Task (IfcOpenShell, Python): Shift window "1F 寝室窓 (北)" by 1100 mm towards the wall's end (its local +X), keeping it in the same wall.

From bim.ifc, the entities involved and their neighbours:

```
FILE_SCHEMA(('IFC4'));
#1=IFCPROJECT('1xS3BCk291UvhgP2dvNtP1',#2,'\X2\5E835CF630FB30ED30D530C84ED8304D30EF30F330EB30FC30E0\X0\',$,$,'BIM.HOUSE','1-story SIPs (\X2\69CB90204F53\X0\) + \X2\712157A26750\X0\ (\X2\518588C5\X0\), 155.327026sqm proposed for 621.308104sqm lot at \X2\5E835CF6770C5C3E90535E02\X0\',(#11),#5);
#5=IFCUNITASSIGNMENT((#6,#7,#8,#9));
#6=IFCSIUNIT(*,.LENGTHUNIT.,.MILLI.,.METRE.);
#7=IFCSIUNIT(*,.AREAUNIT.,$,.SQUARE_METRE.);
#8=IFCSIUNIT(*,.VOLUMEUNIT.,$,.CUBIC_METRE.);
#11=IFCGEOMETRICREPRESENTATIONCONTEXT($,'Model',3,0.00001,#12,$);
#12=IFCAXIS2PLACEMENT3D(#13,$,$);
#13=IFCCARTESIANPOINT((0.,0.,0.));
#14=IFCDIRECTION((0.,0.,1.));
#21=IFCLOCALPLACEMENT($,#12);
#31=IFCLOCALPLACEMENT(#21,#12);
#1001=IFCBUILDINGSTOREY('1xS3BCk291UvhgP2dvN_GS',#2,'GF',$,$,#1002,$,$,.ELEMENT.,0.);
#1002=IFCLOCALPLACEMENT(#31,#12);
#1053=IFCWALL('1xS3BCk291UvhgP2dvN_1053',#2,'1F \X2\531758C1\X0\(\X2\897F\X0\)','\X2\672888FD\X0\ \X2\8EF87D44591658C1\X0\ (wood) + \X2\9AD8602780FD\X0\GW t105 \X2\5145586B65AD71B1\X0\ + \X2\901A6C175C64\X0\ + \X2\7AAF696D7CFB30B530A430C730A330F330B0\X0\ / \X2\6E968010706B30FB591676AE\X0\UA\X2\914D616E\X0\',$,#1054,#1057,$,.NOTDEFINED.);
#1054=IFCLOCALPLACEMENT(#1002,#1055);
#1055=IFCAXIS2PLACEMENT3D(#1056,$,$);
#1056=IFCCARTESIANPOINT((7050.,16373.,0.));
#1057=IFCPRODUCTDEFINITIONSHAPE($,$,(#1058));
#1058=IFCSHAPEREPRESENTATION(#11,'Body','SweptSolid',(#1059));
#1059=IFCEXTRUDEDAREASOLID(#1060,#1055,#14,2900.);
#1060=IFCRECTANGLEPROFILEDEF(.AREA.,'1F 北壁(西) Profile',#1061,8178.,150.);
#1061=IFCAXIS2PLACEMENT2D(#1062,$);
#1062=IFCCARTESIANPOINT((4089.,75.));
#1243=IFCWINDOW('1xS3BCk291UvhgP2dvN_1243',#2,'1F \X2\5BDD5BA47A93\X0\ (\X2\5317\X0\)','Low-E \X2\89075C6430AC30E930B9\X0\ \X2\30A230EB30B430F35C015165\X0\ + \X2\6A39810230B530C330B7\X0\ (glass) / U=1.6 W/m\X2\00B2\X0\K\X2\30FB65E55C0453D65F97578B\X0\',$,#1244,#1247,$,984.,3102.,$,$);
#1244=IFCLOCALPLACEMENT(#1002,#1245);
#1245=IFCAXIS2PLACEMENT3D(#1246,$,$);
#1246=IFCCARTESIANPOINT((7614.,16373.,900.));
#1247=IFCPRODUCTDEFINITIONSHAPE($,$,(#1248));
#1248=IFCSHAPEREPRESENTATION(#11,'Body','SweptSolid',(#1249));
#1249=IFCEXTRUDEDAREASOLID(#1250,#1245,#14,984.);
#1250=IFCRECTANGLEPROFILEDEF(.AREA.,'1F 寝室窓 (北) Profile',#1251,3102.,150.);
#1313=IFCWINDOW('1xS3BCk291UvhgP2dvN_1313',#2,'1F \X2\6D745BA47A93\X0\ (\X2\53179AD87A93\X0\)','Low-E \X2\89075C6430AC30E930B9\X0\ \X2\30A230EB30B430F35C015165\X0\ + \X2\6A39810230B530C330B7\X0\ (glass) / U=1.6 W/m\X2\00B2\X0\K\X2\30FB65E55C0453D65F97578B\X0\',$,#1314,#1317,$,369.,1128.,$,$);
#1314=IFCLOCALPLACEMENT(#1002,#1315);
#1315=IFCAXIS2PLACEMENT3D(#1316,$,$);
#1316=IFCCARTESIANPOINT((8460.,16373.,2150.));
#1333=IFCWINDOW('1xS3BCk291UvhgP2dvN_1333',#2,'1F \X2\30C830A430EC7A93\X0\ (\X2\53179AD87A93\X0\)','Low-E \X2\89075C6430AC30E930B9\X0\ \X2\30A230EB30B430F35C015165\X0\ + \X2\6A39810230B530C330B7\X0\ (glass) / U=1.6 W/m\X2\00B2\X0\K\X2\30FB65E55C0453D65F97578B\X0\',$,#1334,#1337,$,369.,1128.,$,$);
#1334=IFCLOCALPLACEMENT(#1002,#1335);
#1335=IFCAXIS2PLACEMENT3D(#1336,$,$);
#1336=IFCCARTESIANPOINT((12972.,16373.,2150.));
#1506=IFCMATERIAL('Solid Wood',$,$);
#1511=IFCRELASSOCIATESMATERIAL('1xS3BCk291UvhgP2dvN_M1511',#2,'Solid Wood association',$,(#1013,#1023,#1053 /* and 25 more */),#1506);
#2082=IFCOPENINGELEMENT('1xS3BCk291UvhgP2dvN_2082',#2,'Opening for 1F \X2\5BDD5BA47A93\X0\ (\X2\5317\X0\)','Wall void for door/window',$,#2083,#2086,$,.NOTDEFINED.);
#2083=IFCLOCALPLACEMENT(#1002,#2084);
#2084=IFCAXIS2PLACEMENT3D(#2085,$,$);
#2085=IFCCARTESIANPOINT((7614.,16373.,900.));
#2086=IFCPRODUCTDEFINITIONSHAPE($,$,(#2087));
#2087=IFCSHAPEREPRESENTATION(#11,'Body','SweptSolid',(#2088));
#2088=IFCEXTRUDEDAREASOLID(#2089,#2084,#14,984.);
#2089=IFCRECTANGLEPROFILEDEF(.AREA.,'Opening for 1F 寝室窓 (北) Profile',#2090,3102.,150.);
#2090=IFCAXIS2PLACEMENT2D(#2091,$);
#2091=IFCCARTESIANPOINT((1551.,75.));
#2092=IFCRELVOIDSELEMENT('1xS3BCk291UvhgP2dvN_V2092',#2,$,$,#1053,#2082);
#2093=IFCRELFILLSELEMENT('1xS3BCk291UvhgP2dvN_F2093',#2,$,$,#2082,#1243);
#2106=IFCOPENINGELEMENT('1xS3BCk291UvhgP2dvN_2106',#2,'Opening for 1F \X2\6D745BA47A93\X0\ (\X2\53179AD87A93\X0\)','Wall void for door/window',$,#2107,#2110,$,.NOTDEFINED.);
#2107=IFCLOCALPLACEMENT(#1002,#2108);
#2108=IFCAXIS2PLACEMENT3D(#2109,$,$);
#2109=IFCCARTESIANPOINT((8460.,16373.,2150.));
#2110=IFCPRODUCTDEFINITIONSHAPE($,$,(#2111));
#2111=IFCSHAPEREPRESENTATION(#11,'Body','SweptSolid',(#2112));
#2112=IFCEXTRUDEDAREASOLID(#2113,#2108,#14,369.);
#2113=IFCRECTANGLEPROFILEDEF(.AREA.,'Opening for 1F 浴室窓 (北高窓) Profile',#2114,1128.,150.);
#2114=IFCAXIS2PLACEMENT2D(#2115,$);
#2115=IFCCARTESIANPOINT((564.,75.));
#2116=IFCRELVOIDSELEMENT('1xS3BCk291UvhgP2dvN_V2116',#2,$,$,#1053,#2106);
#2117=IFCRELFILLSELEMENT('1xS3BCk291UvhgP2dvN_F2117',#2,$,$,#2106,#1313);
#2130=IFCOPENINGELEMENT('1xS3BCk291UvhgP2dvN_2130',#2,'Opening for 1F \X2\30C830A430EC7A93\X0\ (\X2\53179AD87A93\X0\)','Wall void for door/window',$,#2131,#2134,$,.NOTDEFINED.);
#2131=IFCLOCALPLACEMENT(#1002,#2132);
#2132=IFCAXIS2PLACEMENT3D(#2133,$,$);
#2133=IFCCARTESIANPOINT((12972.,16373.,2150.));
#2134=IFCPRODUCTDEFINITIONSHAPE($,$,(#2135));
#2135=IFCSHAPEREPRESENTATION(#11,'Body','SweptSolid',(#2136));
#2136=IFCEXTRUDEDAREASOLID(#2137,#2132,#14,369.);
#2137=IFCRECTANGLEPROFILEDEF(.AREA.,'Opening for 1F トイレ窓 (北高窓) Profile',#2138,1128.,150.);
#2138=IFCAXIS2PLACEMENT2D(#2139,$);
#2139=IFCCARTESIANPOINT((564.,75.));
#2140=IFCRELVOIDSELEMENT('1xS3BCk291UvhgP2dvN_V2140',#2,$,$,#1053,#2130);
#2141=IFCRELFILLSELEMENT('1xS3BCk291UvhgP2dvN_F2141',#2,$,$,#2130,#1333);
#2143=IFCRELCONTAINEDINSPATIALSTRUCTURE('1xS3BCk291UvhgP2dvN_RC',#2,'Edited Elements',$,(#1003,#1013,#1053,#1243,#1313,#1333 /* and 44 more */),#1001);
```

```python
import ifcopenshell
import ifcopenshell.api.geometry
import ifcopenshell.util.placement
import ifcopenshell.util.unit

model = ifcopenshell.open("bim.ifc")
unit_scale = ifcopenshell.util.unit.calculate_unit_scale(model)

window = model.by_guid("1xS3BCk291UvhgP2dvN_1243")
opening = window.FillsVoids[0].RelatingOpeningElement
wall = opening.VoidsElements[0].RelatingBuildingElement

wall_matrix = ifcopenshell.util.placement.get_local_placement(wall.ObjectPlacement)
shift = wall_matrix[:3, 0] * 1.1 / unit_scale
before = ifcopenshell.util.placement.get_local_placement(window.ObjectPlacement)[:3, 3].copy()

# The window is not placed relative to its opening, so move both.
for product in (opening, window):
    matrix = ifcopenshell.util.placement.get_local_placement(product.ObjectPlacement)
    matrix[:3, 3] += shift
    ifcopenshell.api.geometry.edit_object_placement(model, product=product, matrix=matrix, is_si=False)

after = ifcopenshell.util.placement.get_local_placement(window.ObjectPlacement)[:3, 3]
print("window moved by", (after - before).round(3) + 0.0)

model.write("bim_rev.ifc")
```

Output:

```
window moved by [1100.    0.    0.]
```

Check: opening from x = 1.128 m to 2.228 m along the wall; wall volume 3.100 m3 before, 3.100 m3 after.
